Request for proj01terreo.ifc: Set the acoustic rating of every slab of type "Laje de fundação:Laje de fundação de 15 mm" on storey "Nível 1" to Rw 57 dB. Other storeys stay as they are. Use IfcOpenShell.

First a look at what the model holds.

```python
import ifcopenshell
import ifcopenshell.util.element

model = ifcopenshell.open("proj01terreo.ifc")
print(model.schema)
storey = next(s for s in model.by_type("IfcBuildingStorey") if s.Name == "Nível 1")
slabs = [e for e in ifcopenshell.util.element.get_decomposition(storey) if e.is_a("IfcSlab")]
seen = {}
for e in slabs:
    element_type = ifcopenshell.util.element.get_type(e)
    key = (element_type.Name if element_type != e and element_type else None, ifcopenshell.util.element.get_pset(e, "Pset_SlabCommon", "AcousticRating"))
    seen[key] = seen.get(key, 0) + 1
for (name, value), count in sorted(seen.items(), key=str):
    print(count, "x", name, "|", value)
```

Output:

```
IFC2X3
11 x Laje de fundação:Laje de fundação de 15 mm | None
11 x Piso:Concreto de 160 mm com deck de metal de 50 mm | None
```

```python
import ifcopenshell
import ifcopenshell.api.pset
import ifcopenshell.util.element

model = ifcopenshell.open("proj01terreo.ifc")

storey = next(s for s in model.by_type("IfcBuildingStorey") if s.Name == "Nível 1")
slabs = [e for e in ifcopenshell.util.element.get_decomposition(storey) if e.is_a("IfcSlab")]

count = 0
for e in slabs:
    element_type = ifcopenshell.util.element.get_type(e)
    if element_type in (None, e) or element_type.Name != "Laje de fundação:Laje de fundação de 15 mm":
        continue
    # add_pset returns the element's existing set when there is one.
    pset = ifcopenshell.api.pset.add_pset(model, product=e, name="Pset_SlabCommon")
    ifcopenshell.api.pset.edit_pset(model, pset=pset, properties={"AcousticRating": "Rw 57 dB"})
    count += 1

print(count, "slabs updated")

model.write("proj01terreo_rev.ifc")
```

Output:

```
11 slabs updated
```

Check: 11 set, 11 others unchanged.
